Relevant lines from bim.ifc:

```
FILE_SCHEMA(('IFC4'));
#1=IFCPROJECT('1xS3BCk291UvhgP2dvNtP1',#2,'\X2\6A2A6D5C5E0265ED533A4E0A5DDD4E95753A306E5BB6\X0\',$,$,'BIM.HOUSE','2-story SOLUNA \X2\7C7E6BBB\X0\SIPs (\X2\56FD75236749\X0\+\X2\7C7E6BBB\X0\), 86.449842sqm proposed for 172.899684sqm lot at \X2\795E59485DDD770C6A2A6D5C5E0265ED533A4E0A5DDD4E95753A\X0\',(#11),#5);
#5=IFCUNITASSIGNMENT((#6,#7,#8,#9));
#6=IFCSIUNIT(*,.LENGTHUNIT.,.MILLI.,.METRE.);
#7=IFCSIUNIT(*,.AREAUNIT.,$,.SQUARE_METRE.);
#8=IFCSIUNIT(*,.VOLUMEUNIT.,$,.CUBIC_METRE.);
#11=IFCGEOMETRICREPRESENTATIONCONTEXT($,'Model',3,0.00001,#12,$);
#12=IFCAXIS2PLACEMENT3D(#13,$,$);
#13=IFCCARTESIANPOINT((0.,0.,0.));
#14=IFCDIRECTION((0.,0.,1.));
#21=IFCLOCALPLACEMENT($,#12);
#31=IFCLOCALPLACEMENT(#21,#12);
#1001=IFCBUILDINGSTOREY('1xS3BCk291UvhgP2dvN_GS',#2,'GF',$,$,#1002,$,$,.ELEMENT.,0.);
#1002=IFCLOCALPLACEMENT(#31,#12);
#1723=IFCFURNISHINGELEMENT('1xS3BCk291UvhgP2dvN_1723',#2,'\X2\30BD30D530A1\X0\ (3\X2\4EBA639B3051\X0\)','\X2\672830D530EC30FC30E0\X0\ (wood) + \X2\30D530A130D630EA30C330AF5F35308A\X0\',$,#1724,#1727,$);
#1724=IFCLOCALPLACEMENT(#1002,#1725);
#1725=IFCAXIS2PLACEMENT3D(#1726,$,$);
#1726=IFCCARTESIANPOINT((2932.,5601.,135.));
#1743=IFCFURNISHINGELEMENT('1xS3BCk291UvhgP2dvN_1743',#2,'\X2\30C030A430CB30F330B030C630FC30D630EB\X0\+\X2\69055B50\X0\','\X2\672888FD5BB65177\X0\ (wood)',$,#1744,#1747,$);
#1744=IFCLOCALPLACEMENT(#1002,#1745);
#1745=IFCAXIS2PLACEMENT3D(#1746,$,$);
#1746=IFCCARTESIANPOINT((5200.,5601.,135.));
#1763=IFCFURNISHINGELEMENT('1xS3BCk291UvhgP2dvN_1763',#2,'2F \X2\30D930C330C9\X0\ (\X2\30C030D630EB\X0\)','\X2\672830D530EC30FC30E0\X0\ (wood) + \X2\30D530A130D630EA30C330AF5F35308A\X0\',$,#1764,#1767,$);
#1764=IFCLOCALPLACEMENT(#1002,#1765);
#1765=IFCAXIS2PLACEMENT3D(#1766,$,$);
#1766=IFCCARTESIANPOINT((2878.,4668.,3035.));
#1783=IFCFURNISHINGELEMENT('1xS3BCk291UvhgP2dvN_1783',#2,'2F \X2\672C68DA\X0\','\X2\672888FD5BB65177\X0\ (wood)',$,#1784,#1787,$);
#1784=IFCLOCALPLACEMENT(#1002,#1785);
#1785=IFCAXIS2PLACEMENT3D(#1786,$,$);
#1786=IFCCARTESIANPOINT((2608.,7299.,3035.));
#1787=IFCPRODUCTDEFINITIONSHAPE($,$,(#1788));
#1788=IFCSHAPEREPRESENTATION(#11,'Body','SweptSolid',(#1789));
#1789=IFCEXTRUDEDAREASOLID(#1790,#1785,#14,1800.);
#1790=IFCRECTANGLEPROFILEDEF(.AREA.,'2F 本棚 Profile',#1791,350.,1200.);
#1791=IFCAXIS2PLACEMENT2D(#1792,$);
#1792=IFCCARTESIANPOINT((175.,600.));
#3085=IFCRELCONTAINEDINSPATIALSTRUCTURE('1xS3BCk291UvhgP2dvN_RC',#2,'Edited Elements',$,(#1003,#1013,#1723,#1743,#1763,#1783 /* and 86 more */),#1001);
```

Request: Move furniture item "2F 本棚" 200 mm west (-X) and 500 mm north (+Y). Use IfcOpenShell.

```python
import ifcopenshell
import ifcopenshell.api.geometry
import ifcopenshell.util.placement

model = ifcopenshell.open("bim.ifc")

item = model.by_id(1783)
matrix = ifcopenshell.util.placement.get_local_placement(item.ObjectPlacement)
matrix[0, 3] -= 200.0
matrix[1, 3] += 500.0
ifcopenshell.api.geometry.edit_object_placement(model, product=item, matrix=matrix, is_si=False)

print(ifcopenshell.util.placement.get_local_placement(item.ObjectPlacement).round(3) + 0.0)

model.write("bim_rev.ifc")
```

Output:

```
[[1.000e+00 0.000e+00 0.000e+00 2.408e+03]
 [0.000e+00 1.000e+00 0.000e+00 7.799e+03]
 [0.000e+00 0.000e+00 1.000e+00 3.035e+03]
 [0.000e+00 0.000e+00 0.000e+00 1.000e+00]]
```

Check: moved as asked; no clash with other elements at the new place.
